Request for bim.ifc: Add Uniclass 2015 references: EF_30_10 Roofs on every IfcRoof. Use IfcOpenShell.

First a look at what the model holds.

```python
import ifcopenshell

model = ifcopenshell.open("bim.ifc")
print(model.schema)
print("classifications:", [c.Name for c in model.by_type("IfcClassification")])
for ifc_class in ("IfcDoor", "IfcRoof", "IfcStair", "IfcWall", "IfcWindow"):
    print(ifc_class, len(model.by_type(ifc_class)))
```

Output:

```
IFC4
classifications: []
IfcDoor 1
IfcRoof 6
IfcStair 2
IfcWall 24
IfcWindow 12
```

```python
import ifcopenshell
import ifcopenshell.api.classification

model = ifcopenshell.open("bim.ifc")

system = ifcopenshell.api.classification.add_classification(model, classification="Uniclass 2015")

codes = {
    "IfcRoof": ("EF_30_10", "Roofs"),
}
for ifc_class, (code, name) in codes.items():
    products = model.by_type(ifc_class)
    ifcopenshell.api.classification.add_reference(
        model, products=products, classification=system, identification=code, name=name
    )
    print(code, len(products))

model.write("bim-out.ifc")
```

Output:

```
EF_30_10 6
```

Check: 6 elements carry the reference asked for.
